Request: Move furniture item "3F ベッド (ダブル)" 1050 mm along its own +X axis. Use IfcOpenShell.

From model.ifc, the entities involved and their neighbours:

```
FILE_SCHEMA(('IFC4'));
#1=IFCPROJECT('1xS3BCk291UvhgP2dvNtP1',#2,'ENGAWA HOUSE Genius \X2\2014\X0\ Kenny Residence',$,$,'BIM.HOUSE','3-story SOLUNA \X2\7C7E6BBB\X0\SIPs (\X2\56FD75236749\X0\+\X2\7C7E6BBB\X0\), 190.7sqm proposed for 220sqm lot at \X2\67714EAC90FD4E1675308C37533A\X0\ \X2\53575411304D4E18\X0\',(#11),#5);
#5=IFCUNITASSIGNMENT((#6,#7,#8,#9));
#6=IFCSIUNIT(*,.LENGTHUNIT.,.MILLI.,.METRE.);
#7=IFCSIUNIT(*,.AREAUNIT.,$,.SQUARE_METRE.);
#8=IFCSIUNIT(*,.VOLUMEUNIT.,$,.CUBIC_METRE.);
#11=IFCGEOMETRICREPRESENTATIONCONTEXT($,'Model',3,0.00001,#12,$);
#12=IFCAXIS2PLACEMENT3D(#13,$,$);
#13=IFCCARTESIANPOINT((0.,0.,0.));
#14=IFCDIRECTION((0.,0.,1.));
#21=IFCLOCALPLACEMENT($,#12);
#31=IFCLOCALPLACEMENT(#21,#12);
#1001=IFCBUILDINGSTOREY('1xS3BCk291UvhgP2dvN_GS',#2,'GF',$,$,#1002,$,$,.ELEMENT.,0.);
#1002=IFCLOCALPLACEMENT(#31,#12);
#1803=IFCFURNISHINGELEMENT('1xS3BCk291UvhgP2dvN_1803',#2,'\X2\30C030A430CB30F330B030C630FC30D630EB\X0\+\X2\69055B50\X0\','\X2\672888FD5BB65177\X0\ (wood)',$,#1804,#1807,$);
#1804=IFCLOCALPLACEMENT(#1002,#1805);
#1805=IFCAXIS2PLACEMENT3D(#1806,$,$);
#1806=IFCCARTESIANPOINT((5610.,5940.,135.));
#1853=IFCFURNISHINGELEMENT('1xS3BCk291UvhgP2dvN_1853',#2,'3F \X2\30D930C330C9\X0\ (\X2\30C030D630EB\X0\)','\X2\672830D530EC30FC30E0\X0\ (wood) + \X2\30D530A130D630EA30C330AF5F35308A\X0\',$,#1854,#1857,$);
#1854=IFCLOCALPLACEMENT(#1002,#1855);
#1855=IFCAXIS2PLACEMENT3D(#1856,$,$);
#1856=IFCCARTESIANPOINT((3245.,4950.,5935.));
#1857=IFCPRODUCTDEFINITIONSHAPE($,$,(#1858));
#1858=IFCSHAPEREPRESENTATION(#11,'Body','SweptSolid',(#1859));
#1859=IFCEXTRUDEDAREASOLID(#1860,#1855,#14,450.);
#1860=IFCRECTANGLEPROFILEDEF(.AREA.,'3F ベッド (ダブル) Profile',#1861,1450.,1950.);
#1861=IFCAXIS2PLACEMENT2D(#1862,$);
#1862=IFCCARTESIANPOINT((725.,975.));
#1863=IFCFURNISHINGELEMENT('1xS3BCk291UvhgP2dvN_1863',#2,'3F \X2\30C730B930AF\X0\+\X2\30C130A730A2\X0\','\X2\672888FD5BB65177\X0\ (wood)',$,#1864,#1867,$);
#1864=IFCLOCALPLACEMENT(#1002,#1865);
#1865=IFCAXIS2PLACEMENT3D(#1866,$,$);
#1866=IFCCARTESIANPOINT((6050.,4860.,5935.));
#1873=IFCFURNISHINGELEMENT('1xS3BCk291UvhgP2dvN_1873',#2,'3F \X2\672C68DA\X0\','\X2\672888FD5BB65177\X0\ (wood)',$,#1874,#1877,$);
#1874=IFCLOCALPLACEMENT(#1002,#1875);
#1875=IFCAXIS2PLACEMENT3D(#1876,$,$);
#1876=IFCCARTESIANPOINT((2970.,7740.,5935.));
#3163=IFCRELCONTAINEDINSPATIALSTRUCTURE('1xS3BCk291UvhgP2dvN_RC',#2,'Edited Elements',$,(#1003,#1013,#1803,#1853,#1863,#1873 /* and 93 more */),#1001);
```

```python
import ifcopenshell
import ifcopenshell.api.geometry
import ifcopenshell.util.placement
import ifcopenshell.util.unit

model = ifcopenshell.open("model.ifc")
unit_scale = ifcopenshell.util.unit.calculate_unit_scale(model)

item = model.by_guid("1xS3BCk291UvhgP2dvN_1853")
matrix = ifcopenshell.util.placement.get_local_placement(item.ObjectPlacement)
matrix[:3, 3] += matrix[:3, 0] * 1.05 / unit_scale
ifcopenshell.api.geometry.edit_object_placement(model, product=item, matrix=matrix, is_si=False)

print(ifcopenshell.util.placement.get_local_placement(item.ObjectPlacement).round(3) + 0.0)

model.write("model_updated.ifc")
```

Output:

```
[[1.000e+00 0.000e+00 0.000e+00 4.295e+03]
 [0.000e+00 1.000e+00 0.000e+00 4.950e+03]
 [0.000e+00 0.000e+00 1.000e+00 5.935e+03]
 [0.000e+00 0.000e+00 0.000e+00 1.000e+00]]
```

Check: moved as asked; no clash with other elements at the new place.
